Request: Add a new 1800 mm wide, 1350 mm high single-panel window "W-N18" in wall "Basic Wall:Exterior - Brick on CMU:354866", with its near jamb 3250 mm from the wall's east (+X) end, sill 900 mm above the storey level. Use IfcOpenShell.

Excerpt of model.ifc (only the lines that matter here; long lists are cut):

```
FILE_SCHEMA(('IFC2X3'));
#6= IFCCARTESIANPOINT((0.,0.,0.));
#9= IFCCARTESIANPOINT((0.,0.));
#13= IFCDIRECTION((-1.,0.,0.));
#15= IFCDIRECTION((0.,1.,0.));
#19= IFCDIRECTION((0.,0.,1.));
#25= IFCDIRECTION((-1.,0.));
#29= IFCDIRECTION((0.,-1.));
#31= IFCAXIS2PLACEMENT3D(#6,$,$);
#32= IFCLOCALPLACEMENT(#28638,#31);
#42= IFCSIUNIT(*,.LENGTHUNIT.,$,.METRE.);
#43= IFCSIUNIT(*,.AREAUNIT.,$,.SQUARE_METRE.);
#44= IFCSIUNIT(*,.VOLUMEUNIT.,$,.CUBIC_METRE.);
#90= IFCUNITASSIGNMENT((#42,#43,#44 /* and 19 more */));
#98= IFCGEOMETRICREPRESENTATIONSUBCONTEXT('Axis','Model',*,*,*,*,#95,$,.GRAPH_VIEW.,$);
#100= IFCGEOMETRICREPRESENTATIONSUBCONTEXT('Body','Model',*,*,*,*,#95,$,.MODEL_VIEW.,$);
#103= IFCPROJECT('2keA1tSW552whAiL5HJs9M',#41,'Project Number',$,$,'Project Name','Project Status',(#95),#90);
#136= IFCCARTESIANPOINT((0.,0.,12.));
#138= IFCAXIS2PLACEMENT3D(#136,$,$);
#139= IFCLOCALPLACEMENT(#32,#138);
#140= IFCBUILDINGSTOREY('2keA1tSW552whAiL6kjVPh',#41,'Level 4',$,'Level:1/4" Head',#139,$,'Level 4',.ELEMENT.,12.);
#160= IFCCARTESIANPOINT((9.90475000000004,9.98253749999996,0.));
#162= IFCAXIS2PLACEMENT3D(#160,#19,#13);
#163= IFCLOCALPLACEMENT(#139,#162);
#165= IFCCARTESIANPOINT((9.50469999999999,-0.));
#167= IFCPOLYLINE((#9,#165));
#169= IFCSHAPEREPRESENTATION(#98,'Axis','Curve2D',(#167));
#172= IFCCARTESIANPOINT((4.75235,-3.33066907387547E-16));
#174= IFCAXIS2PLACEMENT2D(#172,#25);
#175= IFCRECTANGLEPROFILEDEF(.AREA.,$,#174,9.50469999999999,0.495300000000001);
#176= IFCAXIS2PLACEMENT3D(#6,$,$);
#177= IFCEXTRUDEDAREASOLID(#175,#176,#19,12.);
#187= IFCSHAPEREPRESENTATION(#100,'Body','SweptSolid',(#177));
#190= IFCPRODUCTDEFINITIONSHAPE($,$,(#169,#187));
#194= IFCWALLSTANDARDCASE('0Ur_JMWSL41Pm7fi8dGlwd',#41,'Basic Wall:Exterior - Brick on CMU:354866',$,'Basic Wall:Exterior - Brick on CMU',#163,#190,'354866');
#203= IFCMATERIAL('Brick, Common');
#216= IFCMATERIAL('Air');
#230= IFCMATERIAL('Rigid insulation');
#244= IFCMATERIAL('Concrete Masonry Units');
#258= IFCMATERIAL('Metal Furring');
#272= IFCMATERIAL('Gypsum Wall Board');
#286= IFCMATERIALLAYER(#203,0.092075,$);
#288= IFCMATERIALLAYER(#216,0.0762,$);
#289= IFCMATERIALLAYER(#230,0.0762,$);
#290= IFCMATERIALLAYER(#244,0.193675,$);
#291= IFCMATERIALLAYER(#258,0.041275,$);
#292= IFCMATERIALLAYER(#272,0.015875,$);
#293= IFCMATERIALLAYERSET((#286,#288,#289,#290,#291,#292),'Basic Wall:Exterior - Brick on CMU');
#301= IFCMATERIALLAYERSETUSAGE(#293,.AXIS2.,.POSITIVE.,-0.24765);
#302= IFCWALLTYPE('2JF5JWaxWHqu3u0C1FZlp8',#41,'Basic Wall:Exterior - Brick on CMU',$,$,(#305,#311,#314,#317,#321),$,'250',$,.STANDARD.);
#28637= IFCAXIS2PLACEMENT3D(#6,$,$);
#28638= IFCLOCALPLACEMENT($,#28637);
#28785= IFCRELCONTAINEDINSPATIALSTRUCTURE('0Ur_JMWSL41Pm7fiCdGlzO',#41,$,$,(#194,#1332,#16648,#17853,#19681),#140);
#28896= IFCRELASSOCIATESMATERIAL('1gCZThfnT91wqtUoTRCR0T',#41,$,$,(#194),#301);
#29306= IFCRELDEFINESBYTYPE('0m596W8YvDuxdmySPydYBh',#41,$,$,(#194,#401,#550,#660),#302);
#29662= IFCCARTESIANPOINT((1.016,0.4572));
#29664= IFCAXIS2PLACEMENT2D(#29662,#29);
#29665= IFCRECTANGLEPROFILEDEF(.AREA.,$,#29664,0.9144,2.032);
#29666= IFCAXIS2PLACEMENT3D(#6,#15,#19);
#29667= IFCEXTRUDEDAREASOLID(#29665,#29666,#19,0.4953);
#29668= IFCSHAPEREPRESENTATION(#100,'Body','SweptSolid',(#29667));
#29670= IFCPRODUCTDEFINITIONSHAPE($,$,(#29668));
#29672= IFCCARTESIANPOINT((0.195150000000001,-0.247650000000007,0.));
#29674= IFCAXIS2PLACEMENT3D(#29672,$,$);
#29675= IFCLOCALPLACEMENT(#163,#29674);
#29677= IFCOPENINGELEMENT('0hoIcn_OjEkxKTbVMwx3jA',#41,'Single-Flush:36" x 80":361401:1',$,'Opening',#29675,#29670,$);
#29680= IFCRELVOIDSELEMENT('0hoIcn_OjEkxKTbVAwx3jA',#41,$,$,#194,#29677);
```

```python
import numpy as np
import ifcopenshell
import ifcopenshell.api.feature
import ifcopenshell.api.geometry
import ifcopenshell.api.root
import ifcopenshell.api.spatial
import ifcopenshell.api.type
import ifcopenshell.geom
import ifcopenshell.util.element
import ifcopenshell.util.placement
import ifcopenshell.util.representation
import ifcopenshell.util.shape
import ifcopenshell.util.unit

model = ifcopenshell.open("model.ifc")
unit_scale = ifcopenshell.util.unit.calculate_unit_scale(model)
settings = ifcopenshell.geom.settings()


def volume(element):
    """Net volume in cubic metres, openings subtracted."""
    shape = ifcopenshell.geom.create_shape(settings, element)
    return ifcopenshell.util.shape.get_volume(shape.geometry)


wall = model.by_id(194)
storey = ifcopenshell.util.element.get_container(wall, ifc_class="IfcBuildingStorey")
context = ifcopenshell.util.representation.get_context(model, "Model", "Body", "MODEL_VIEW")
before = volume(wall)

width, height, from_end, sill = 1.8, 1.35, 3.25, 0.9  # metres

# The wall runs along its own X axis, and the end named is its -X end.
wall_shape = ifcopenshell.geom.create_shape(settings, wall)
x, y, z = ifcopenshell.util.shape.get_vertices(wall_shape.geometry).T
start = x.min() + from_end
face, thickness = float(y.min()), float(y.max() - y.min())
wall_matrix = ifcopenshell.util.placement.get_local_placement(wall.ObjectPlacement)
level = ifcopenshell.util.placement.get_local_placement(storey.ObjectPlacement)[2, 3]


def in_wall(x, y):
    """Placement at x, y metres in the wall's axes, at sill height."""
    matrix = wall_matrix.copy()
    matrix[:, 3] = wall_matrix @ np.array([x / unit_scale, y / unit_scale, 0.0, 1.0])
    matrix[2, 3] = level + sill / unit_scale
    return matrix


# Opening: a box that overshoots both wall faces by 50 mm.
opening = ifcopenshell.api.root.create_entity(model, ifc_class="IfcOpeningElement")
box = ifcopenshell.api.geometry.add_wall_representation(
    model, context=context, length=width, height=height, thickness=thickness + 0.1
)
ifcopenshell.api.geometry.assign_representation(model, product=opening, representation=box)
ifcopenshell.api.geometry.edit_object_placement(model, product=opening, matrix=in_wall(start, face - 0.05), is_si=False)
ifcopenshell.api.feature.add_feature(model, feature=opening, element=wall)

window = ifcopenshell.api.root.create_entity(model, ifc_class="IfcWindow", name="W-N18")
window.OverallWidth, window.OverallHeight = width / unit_scale, height / unit_scale
body = ifcopenshell.api.geometry.add_window_representation(
    model,
    context=context,
    overall_width=window.OverallWidth,
    overall_height=window.OverallHeight,
    partition_type="SINGLE_PANEL",
)
ifcopenshell.api.geometry.assign_representation(model, product=window, representation=body)
ifcopenshell.api.spatial.assign_container(model, products=[window], relating_structure=storey)
fills = ifcopenshell.api.feature.add_filling(model, opening=opening, element=window)
fills.OwnerHistory = window.OwnerHistory  # required in IFC2X3

# IFC2X3 keeps the operation on the window style.
style = ifcopenshell.api.root.create_entity(model, ifc_class="IfcWindowStyle", name="W-N18")
style.OperationType, style.ConstructionType = "SINGLE_PANEL", "NOTDEFINED"
style.ParameterTakesPrecedence = style.Sizeable = False
ifcopenshell.api.type.assign_type(model, related_objects=[window], relating_type=style)

# Centre the window in the wall's thickness.
ifcopenshell.api.geometry.edit_object_placement(model, product=window, matrix=in_wall(start, face), is_si=False)
window_shape = ifcopenshell.geom.create_shape(settings, window)
depth = ifcopenshell.util.shape.get_vertices(window_shape.geometry)[:, 1]
offset = face + thickness / 2 - (depth.min() + depth.max()) / 2
ifcopenshell.api.geometry.edit_object_placement(model, product=window, matrix=in_wall(start, offset), is_si=False)

after = volume(wall)

print(f"wall volume {before:.3f} -> {after:.3f} m3")

model.write("model_edited.ifc")
```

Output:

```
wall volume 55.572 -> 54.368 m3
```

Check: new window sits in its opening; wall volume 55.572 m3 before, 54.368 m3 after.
